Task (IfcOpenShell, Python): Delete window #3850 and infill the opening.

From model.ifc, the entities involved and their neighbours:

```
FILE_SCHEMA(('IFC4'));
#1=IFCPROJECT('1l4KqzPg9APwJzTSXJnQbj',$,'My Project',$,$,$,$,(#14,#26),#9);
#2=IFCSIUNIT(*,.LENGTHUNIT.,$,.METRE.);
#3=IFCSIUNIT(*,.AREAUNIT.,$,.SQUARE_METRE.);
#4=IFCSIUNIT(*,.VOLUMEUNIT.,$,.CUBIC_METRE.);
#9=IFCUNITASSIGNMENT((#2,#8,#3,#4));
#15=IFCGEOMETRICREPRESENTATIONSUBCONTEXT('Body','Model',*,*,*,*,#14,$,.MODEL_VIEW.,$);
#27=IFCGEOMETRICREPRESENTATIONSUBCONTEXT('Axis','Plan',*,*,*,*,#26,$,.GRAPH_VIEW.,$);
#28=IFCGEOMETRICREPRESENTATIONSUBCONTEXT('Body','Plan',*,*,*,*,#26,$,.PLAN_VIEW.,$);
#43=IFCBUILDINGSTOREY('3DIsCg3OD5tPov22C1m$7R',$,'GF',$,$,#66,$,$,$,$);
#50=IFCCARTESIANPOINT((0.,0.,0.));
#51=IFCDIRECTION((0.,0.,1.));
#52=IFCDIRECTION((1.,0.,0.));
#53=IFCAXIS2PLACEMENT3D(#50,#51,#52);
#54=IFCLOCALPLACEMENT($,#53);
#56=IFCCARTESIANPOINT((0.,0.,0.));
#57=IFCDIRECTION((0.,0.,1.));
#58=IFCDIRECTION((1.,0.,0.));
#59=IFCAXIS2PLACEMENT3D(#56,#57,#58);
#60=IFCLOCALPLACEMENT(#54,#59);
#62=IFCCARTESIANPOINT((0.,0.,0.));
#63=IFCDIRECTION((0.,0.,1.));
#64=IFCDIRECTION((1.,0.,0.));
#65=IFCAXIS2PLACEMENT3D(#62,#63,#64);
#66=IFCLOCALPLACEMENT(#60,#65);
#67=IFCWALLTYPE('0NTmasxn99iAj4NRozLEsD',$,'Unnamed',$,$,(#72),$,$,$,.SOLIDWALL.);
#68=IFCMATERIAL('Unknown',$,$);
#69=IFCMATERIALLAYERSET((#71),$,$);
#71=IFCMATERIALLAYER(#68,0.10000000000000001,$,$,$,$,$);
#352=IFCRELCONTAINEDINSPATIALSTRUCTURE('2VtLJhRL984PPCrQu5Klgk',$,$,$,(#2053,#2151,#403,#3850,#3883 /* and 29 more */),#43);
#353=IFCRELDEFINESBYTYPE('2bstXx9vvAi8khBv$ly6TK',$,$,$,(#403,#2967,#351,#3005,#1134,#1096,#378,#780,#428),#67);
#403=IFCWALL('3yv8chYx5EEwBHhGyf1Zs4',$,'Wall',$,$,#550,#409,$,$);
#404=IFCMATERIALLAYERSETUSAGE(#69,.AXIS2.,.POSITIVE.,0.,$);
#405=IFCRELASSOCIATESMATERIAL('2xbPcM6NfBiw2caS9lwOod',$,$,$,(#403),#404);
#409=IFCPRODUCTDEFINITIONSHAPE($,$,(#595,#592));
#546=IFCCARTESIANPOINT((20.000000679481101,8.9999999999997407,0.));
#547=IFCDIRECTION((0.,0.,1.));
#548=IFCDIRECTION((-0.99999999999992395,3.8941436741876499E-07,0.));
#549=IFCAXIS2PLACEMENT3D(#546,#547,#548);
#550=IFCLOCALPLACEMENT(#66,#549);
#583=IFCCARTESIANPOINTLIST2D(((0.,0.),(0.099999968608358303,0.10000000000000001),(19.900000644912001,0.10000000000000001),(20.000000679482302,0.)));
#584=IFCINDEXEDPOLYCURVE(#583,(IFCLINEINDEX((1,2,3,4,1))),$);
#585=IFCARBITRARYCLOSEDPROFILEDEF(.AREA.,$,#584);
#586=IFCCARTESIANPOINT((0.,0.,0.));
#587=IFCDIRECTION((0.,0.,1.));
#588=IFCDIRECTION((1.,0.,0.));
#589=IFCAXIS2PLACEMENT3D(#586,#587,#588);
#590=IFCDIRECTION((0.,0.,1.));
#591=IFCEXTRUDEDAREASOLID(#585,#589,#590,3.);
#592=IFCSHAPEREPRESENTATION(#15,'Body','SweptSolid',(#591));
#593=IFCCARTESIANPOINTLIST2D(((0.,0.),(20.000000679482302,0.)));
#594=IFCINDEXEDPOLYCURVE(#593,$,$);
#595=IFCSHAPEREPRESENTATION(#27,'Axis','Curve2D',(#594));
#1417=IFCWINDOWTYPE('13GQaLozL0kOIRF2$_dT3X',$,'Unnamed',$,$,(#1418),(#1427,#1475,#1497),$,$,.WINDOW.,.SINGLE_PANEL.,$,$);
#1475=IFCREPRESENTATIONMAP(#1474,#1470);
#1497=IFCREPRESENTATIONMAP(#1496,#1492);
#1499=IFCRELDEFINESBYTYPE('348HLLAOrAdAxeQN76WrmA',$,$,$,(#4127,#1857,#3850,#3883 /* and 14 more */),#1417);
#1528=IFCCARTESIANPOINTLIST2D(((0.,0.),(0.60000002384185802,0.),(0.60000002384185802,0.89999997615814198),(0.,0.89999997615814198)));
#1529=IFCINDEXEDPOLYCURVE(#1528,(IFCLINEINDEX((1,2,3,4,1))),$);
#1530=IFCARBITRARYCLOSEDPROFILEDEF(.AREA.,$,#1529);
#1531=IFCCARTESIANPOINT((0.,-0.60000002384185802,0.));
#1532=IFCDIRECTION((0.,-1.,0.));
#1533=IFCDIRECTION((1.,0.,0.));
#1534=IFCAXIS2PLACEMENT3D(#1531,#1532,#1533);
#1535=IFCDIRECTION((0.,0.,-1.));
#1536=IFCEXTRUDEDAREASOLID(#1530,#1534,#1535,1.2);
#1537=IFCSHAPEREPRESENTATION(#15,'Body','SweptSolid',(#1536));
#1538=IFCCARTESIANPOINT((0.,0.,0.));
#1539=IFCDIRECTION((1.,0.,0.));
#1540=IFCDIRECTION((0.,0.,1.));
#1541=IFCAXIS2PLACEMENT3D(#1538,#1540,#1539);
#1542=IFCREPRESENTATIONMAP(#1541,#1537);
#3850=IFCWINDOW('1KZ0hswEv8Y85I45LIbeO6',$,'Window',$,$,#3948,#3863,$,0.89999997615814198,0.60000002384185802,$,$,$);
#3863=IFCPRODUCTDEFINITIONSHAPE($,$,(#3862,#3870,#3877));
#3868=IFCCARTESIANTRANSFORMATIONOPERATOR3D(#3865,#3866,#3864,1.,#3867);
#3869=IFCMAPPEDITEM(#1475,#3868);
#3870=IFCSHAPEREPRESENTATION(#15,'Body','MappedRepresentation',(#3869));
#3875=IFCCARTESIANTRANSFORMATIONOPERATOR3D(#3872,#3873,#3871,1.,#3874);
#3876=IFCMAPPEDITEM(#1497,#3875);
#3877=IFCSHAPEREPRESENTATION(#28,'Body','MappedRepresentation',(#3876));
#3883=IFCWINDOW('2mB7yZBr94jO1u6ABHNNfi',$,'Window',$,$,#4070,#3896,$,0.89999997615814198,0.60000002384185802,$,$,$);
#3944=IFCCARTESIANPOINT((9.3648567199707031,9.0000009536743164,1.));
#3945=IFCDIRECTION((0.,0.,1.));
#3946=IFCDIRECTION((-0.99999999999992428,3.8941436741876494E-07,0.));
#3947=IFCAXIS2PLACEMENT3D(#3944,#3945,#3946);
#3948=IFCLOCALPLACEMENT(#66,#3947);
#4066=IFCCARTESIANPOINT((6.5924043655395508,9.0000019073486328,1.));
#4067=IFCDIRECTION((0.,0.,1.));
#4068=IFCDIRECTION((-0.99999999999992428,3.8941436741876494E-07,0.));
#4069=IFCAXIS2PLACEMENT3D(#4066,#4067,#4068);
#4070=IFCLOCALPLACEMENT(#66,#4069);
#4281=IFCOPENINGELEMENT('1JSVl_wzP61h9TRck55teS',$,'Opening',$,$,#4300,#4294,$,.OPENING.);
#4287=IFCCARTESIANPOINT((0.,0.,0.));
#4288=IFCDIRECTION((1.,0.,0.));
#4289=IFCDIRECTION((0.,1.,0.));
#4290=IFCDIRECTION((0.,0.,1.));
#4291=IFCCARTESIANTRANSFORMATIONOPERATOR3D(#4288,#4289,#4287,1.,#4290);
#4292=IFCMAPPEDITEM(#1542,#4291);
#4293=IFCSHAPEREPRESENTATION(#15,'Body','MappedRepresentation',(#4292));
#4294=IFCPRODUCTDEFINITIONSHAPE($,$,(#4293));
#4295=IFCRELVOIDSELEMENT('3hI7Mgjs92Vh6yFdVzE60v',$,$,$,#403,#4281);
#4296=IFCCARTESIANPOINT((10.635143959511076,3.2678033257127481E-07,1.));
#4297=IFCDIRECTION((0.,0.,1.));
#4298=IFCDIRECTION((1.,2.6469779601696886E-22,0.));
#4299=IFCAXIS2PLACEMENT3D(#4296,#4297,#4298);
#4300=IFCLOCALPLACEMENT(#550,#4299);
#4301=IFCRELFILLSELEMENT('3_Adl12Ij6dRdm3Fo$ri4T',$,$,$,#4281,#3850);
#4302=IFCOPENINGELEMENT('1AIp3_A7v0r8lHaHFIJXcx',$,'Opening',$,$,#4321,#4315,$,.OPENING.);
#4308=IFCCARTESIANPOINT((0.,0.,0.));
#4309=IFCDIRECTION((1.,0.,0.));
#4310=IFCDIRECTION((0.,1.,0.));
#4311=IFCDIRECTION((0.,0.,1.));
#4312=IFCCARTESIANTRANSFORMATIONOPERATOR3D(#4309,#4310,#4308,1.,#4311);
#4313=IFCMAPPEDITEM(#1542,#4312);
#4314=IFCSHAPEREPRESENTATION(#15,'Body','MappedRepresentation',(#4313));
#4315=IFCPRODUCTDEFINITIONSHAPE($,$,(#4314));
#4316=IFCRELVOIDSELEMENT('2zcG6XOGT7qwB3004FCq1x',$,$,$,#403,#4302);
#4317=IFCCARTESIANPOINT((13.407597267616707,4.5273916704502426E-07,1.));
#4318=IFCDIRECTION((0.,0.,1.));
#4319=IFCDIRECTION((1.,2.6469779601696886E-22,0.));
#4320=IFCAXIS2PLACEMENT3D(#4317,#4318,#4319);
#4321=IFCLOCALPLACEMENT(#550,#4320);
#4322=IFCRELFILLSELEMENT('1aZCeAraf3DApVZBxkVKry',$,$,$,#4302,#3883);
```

```python
import ifcopenshell
import ifcopenshell.api.feature
import ifcopenshell.api.root
import ifcopenshell.geom
import ifcopenshell.util.shape

model = ifcopenshell.open("model.ifc")
settings = ifcopenshell.geom.settings()


def volume(element):
    """Net volume in cubic metres, openings subtracted."""
    shape = ifcopenshell.geom.create_shape(settings, element)
    return ifcopenshell.util.shape.get_volume(shape.geometry)


window = model.by_guid("1KZ0hswEv8Y85I45LIbeO6")
opening = window.FillsVoids[0].RelatingOpeningElement
wall = opening.VoidsElements[0].RelatingBuildingElement
before = volume(wall)

ifcopenshell.api.root.remove_product(model, product=window)
ifcopenshell.api.feature.remove_feature(model, feature=opening)

after = volume(wall)

print(f"wall volume {before:.3f} -> {after:.3f} m3")

model.write("model_rev.ifc")
```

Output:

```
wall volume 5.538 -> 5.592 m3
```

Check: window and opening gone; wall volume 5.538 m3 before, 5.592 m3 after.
